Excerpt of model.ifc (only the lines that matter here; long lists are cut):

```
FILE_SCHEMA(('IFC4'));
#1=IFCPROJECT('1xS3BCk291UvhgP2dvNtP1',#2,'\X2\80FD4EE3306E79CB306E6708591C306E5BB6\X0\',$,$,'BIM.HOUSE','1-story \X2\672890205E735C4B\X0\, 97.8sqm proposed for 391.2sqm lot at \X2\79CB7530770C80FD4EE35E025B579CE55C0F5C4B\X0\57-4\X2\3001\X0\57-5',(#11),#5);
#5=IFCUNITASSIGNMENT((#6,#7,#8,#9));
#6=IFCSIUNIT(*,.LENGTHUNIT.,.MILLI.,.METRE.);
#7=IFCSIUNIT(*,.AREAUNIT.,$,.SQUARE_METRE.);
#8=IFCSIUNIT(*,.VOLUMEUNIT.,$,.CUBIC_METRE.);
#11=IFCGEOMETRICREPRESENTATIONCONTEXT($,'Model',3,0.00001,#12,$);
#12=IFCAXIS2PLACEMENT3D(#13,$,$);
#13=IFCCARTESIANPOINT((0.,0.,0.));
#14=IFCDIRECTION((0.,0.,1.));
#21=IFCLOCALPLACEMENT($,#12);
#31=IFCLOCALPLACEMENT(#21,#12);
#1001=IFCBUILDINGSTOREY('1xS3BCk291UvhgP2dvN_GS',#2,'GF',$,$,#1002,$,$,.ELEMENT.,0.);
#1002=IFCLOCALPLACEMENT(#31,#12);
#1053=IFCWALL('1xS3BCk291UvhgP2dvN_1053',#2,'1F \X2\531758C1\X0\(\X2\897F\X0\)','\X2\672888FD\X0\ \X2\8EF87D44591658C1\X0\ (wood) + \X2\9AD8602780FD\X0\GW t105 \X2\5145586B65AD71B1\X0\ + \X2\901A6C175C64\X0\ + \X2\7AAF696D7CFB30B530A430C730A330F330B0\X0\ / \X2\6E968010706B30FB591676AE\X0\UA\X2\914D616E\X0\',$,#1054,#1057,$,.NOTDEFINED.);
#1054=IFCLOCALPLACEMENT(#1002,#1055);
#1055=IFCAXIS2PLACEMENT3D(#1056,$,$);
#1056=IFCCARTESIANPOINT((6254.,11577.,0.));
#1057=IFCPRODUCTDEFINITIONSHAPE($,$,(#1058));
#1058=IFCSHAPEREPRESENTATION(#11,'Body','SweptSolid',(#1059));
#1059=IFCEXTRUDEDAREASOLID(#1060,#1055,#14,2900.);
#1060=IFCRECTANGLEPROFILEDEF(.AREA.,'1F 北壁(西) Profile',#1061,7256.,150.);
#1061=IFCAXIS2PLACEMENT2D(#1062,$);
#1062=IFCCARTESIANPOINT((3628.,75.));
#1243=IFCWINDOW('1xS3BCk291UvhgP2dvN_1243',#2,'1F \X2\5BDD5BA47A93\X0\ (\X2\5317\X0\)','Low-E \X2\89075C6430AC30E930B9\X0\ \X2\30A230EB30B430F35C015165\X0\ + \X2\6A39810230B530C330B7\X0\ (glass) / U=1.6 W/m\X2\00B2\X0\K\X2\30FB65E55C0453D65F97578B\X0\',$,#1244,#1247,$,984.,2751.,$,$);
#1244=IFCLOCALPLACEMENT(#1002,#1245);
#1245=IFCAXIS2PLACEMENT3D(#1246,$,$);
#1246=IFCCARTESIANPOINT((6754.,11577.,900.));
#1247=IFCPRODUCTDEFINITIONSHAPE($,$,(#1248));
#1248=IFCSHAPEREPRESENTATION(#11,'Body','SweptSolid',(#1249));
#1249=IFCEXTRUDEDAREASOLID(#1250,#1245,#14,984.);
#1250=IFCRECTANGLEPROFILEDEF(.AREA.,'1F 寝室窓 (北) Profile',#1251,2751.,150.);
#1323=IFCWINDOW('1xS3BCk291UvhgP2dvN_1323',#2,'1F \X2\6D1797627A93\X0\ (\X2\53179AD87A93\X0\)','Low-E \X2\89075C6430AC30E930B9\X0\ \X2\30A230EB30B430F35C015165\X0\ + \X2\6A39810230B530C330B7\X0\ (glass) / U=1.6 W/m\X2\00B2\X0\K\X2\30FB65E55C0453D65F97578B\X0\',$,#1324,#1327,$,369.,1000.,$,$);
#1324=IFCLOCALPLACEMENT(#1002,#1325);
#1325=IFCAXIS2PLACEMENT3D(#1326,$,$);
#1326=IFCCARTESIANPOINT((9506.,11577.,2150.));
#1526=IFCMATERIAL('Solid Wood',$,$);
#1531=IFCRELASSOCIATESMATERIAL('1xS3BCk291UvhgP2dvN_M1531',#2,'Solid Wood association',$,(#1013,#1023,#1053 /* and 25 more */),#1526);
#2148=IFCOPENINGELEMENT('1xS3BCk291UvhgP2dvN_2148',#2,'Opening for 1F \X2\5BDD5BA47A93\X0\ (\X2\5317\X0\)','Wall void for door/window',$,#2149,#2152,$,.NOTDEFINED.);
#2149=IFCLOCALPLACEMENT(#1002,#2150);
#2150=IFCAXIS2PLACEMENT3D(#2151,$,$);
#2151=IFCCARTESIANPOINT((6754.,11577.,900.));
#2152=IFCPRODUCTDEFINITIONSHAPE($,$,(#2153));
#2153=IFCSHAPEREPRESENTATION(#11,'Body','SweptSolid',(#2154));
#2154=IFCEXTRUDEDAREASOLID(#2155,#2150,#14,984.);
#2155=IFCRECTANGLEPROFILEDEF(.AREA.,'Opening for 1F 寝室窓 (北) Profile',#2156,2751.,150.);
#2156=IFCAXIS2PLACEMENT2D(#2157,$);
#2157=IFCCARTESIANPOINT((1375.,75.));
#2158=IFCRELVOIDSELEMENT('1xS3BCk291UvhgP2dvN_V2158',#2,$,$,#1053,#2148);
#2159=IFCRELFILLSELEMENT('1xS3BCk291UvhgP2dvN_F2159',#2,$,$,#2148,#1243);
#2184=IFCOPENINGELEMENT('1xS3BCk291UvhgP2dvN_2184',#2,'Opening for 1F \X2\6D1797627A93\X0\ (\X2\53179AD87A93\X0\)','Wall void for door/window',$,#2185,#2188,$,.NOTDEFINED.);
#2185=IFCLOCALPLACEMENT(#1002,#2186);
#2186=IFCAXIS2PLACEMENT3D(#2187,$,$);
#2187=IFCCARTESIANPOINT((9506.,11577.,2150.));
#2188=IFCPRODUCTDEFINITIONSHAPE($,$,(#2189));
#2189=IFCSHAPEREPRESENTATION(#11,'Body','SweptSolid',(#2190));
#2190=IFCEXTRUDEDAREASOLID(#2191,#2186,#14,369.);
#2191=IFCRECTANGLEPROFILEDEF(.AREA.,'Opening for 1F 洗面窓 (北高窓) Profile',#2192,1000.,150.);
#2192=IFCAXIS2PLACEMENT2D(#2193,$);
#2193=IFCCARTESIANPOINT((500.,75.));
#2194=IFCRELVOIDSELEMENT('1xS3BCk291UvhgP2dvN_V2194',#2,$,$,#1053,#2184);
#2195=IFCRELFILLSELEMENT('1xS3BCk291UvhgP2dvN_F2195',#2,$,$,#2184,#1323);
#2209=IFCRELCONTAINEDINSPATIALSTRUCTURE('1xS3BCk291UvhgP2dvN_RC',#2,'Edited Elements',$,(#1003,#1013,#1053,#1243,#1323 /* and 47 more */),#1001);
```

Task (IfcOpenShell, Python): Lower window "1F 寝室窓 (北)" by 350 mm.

```python
import numpy as np
import ifcopenshell
import ifcopenshell.api.geometry
import ifcopenshell.util.placement
import ifcopenshell.util.unit

model = ifcopenshell.open("model.ifc")
unit_scale = ifcopenshell.util.unit.calculate_unit_scale(model)

window = model.by_guid("1xS3BCk291UvhgP2dvN_1243")
opening = window.FillsVoids[0].RelatingOpeningElement
dz = -0.35 / unit_scale

shift = np.array([0.0, 0.0, dz])
# The window is not placed relative to its opening, so move both.
for product in (opening, window):
    matrix = ifcopenshell.util.placement.get_local_placement(product.ObjectPlacement)
    matrix[:3, 3] += shift
    ifcopenshell.api.geometry.edit_object_placement(model, product=product, matrix=matrix, is_si=False)

print(f"moved by {dz * unit_scale:+.3f} m")

model.write("model_rev.ifc")
```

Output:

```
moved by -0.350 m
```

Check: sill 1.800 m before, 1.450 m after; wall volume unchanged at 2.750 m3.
